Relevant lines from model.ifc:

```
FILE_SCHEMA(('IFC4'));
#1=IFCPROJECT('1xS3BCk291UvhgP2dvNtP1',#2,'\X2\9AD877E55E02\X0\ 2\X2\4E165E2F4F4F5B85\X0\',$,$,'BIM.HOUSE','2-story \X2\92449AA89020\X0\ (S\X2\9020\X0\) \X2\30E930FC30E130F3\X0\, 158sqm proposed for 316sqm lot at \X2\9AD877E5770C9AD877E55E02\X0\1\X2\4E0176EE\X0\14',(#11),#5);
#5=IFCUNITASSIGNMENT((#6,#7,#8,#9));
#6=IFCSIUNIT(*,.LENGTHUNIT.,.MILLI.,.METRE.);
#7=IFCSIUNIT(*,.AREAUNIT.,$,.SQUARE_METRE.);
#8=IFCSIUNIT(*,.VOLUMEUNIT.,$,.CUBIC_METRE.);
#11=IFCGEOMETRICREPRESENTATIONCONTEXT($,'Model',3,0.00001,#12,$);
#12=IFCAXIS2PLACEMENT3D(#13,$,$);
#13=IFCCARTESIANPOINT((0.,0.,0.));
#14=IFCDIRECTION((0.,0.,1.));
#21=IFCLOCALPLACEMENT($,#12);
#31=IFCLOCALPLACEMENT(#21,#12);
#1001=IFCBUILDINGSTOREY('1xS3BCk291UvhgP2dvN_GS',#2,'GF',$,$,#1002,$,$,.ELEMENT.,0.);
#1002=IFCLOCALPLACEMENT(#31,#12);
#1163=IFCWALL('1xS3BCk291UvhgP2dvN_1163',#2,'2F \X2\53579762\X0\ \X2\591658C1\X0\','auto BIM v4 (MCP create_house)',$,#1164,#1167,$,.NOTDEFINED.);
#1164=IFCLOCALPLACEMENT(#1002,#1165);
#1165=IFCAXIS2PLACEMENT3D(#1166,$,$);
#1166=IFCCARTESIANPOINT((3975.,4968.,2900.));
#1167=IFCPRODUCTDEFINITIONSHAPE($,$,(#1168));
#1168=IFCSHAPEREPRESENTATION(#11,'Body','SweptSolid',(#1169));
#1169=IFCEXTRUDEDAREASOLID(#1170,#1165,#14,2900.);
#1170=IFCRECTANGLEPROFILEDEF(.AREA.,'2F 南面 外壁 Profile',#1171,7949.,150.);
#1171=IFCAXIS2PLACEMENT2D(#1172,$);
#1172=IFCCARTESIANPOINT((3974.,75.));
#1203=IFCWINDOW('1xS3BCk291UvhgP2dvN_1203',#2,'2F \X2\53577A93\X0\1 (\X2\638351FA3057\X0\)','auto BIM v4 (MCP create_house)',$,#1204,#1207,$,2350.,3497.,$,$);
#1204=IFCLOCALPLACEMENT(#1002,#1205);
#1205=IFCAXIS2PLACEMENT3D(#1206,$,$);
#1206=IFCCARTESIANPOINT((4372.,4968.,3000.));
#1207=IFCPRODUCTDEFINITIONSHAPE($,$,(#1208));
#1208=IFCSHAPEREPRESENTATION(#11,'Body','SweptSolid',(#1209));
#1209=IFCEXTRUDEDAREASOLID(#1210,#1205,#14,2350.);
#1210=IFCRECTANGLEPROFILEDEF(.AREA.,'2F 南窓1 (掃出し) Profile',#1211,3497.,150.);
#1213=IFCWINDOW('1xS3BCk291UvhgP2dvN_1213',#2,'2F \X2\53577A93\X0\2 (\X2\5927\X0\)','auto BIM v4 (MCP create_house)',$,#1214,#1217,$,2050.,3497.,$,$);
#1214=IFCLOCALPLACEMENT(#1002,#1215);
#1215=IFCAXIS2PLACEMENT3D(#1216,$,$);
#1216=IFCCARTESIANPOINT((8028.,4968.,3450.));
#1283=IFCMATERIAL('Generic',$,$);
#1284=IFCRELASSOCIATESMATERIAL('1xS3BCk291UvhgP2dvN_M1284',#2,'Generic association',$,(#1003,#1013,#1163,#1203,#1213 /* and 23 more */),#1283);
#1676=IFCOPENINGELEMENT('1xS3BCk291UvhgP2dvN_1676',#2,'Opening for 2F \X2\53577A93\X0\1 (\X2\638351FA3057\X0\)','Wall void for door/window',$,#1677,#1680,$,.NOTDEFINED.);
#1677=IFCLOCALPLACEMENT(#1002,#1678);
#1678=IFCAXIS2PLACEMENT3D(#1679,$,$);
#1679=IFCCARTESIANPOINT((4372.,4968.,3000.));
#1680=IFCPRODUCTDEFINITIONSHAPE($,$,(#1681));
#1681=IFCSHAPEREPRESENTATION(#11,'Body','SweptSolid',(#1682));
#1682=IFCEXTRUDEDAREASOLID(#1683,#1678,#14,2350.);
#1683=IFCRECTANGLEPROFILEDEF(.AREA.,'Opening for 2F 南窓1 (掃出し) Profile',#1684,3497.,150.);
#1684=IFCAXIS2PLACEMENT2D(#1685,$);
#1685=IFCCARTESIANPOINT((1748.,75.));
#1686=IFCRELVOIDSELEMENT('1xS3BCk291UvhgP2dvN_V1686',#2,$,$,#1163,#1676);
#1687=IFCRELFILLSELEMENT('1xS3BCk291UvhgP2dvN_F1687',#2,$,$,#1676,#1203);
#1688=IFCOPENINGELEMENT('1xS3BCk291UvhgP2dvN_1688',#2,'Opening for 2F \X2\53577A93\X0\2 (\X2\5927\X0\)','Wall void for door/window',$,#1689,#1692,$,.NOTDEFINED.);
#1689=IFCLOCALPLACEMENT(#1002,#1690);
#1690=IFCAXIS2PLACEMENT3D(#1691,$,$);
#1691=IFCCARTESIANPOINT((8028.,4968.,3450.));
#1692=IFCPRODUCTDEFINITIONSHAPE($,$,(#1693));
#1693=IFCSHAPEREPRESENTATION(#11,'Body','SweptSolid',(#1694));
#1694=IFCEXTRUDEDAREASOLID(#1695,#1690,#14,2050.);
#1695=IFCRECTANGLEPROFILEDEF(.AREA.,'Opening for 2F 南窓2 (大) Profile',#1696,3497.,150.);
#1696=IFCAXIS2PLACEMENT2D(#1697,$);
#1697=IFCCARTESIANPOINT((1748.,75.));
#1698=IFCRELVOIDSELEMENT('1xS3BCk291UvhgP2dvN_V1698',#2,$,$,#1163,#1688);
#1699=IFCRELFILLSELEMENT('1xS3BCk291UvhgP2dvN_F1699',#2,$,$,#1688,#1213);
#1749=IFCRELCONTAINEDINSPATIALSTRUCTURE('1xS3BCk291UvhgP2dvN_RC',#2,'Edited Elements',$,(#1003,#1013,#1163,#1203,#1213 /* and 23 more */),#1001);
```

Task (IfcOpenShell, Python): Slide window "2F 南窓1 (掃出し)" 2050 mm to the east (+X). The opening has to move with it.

```python
import ifcopenshell
import ifcopenshell.api.geometry
import ifcopenshell.util.placement

model = ifcopenshell.open("model.ifc")

window = model.by_id(1203)
opening = window.FillsVoids[0].RelatingOpeningElement
wall = opening.VoidsElements[0].RelatingBuildingElement

wall_matrix = ifcopenshell.util.placement.get_local_placement(wall.ObjectPlacement)
shift = wall_matrix[:3, 0] * 2050.0
before = ifcopenshell.util.placement.get_local_placement(window.ObjectPlacement)[:3, 3].copy()

# The window is not placed relative to its opening, so move both.
for product in (opening, window):
    matrix = ifcopenshell.util.placement.get_local_placement(product.ObjectPlacement)
    matrix[:3, 3] += shift
    ifcopenshell.api.geometry.edit_object_placement(model, product=product, matrix=matrix, is_si=False)

after = ifcopenshell.util.placement.get_local_placement(window.ObjectPlacement)[:3, 3]
print("window moved by", (after - before).round(3) + 0.0)

model.write("model-out.ifc")
```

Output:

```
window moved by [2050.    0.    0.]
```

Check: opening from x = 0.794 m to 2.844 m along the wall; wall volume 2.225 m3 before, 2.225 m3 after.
